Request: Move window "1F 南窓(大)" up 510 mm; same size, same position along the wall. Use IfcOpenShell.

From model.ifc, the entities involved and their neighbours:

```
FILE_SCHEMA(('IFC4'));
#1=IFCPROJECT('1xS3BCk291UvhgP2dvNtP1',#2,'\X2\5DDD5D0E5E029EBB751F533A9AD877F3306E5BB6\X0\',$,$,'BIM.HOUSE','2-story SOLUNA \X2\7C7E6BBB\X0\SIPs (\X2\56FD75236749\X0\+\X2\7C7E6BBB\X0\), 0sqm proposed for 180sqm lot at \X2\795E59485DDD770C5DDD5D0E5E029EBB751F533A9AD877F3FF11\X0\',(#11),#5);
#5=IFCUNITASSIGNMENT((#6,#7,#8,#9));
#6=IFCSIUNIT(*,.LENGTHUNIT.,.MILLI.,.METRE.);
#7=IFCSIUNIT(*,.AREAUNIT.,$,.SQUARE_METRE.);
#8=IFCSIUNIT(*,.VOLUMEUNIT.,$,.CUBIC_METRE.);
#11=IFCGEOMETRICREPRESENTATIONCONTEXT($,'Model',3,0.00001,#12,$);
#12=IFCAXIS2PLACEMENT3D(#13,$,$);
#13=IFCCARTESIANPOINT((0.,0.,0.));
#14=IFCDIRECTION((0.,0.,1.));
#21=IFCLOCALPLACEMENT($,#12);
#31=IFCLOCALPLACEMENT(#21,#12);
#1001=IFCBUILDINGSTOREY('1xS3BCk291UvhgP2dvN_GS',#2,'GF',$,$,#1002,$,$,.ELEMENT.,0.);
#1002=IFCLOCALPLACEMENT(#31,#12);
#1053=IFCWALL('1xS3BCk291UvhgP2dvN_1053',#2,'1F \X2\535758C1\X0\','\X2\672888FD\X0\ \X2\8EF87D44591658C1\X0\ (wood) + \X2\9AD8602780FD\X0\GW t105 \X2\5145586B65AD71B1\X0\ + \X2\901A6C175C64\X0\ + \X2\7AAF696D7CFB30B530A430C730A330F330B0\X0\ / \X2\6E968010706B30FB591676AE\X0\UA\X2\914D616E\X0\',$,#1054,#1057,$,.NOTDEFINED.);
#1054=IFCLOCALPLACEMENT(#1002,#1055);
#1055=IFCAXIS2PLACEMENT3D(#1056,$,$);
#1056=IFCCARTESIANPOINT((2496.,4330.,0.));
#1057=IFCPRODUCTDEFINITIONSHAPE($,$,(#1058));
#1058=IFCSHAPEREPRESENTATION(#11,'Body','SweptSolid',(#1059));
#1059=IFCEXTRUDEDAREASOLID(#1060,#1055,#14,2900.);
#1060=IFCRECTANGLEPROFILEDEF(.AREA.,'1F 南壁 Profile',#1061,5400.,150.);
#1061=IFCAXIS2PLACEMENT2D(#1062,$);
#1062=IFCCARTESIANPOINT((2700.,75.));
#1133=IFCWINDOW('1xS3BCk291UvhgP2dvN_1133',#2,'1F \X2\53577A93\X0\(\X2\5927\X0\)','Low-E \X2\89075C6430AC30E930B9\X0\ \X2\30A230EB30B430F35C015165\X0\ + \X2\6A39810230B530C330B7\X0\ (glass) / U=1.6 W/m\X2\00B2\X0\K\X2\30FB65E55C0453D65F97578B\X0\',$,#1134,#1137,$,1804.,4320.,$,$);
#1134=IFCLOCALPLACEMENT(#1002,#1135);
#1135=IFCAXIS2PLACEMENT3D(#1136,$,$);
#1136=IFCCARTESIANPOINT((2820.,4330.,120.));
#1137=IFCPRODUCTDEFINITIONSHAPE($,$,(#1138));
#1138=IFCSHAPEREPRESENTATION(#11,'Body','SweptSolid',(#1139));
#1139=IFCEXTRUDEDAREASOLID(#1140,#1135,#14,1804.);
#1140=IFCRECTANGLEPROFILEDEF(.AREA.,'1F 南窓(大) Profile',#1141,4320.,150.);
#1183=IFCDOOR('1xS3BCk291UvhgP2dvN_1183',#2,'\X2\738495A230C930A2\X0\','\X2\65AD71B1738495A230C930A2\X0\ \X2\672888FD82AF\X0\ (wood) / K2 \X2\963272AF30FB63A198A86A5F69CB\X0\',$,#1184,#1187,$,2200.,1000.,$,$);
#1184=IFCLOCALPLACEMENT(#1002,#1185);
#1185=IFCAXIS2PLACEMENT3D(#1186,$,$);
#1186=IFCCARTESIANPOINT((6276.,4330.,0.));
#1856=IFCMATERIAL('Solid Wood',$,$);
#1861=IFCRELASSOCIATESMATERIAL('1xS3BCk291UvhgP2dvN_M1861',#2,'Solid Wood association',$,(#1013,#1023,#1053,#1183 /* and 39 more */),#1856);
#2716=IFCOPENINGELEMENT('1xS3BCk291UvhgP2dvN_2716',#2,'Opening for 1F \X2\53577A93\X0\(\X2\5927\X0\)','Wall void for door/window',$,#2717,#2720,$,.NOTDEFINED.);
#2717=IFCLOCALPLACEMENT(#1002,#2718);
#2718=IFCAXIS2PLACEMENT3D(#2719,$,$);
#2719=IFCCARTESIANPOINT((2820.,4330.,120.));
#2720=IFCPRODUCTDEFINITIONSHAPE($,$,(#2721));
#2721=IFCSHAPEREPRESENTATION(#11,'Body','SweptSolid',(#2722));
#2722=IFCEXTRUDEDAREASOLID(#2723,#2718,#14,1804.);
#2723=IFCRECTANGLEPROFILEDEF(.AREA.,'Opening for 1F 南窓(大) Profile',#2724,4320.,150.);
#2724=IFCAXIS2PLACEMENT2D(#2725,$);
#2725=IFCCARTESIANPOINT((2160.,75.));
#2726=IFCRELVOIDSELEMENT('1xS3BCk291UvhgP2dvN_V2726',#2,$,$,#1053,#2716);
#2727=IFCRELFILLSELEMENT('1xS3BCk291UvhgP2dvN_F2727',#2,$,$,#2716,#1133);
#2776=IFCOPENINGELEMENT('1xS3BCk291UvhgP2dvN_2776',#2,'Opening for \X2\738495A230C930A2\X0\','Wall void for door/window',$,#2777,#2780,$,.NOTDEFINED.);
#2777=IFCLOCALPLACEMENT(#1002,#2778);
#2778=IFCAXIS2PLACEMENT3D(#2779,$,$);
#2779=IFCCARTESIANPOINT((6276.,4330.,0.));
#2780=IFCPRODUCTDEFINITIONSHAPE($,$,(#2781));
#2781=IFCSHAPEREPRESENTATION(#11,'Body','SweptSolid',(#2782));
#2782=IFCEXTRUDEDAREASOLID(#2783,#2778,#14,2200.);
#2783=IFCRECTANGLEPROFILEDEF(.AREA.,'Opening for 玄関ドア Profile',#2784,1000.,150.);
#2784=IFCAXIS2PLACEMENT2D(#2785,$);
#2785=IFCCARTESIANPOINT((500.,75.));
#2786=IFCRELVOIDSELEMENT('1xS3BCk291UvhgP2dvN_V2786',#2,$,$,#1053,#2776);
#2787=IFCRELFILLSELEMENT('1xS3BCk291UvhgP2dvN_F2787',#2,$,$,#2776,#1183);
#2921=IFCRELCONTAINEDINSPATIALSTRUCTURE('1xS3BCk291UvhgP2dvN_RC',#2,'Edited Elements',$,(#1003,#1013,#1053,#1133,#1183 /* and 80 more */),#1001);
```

```python
import numpy as np
import ifcopenshell
import ifcopenshell.api.geometry
import ifcopenshell.util.placement
import ifcopenshell.util.unit

model = ifcopenshell.open("model.ifc")
unit_scale = ifcopenshell.util.unit.calculate_unit_scale(model)

window = model.by_id(1133)
opening = window.FillsVoids[0].RelatingOpeningElement
dz = 0.51 / unit_scale

shift = np.array([0.0, 0.0, dz])
# The window is not placed relative to its opening, so move both.
for product in (opening, window):
    matrix = ifcopenshell.util.placement.get_local_placement(product.ObjectPlacement)
    matrix[:3, 3] += shift
    ifcopenshell.api.geometry.edit_object_placement(model, product=product, matrix=matrix, is_si=False)

print(f"moved by {dz * unit_scale:+.3f} m")

model.write("model_rev.ifc")
```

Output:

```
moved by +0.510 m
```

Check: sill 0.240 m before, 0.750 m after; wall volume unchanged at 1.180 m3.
